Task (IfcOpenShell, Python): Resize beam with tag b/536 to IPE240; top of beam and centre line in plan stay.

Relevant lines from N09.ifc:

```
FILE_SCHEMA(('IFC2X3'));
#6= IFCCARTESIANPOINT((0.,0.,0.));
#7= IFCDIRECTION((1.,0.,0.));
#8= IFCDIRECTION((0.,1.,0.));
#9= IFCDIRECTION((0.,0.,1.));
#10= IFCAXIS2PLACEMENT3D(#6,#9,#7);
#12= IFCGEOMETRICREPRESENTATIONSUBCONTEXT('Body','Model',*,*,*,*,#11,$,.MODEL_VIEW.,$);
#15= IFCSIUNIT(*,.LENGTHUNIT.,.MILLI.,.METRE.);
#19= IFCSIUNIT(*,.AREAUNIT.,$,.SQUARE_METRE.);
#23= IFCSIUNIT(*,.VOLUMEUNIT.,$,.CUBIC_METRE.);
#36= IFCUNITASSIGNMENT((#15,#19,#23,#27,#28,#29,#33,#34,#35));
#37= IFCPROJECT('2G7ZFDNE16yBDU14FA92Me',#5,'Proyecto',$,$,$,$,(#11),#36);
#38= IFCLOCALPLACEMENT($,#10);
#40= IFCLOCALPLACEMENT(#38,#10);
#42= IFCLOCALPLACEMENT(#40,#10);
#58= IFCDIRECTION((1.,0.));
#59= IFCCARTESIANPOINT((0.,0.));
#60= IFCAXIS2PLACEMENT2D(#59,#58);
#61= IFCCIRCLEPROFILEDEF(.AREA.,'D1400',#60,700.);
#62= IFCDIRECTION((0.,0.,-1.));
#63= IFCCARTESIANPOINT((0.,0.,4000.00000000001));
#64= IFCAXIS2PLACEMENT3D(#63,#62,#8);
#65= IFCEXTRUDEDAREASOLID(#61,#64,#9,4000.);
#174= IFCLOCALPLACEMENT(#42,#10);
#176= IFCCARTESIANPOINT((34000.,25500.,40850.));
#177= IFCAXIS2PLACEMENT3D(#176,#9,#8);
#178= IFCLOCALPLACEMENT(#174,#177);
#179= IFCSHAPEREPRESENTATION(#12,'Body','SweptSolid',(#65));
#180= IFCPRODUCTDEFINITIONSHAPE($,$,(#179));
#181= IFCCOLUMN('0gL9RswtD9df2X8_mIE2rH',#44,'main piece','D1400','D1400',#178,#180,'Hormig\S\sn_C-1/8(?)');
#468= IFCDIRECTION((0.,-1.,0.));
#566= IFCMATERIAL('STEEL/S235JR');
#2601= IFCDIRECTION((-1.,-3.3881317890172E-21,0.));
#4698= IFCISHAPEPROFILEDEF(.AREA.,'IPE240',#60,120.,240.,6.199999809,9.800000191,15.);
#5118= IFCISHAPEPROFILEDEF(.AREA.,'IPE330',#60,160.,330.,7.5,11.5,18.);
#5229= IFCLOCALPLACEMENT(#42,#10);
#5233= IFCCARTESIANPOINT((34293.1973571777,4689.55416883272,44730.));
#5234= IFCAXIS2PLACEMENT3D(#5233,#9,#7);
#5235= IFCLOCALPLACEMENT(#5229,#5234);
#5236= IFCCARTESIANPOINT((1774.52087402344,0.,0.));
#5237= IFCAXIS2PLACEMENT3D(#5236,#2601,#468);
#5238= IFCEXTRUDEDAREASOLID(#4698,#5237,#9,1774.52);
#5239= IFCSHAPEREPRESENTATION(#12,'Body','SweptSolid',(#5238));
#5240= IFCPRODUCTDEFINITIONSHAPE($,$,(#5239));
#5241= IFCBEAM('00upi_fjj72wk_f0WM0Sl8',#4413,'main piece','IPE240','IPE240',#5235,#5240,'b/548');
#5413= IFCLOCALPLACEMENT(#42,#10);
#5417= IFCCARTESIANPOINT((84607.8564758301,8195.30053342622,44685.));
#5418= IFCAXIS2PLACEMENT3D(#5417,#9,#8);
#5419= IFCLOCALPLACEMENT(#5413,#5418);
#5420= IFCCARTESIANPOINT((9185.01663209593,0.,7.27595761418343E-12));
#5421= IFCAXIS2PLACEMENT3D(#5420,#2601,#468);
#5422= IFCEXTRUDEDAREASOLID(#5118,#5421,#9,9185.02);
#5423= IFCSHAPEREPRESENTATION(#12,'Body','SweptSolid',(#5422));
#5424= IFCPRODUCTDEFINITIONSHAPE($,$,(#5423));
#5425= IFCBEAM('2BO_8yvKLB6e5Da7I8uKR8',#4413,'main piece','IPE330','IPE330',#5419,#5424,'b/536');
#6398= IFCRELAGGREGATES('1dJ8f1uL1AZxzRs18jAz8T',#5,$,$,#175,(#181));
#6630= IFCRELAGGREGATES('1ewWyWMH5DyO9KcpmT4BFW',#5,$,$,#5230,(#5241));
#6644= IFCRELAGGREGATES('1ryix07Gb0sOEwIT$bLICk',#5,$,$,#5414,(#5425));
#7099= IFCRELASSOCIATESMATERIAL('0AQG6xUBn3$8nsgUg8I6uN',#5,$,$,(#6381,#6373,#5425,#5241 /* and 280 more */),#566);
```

```python
import ifcopenshell
import ifcopenshell.util.element
import ifcopenshell.util.representation

model = ifcopenshell.open("N09.ifc")

member = model.by_guid("2BO_8yvKLB6e5Da7I8uKR8")
source = next(p for p in model.by_type("IfcIShapeProfileDef") if p.ProfileName == "IPE240")

body = ifcopenshell.util.representation.get_representation(member, "Model", "Body")
solid = body.Items[0]
old_profile = solid.SweptArea

# Copy the section's sizes but keep this member's own profile position.
profile = ifcopenshell.util.element.copy(model, source)
# Profiles are centred, so shift by half the change in depth to hold the top.
shift = (old_profile.OverallDepth - profile.OverallDepth) / 2
x, y = old_profile.Position.Location.Coordinates
up = (0.0, 1.0)  # upwards, in the solid's own plane
location = model.createIfcCartesianPoint((x + up[0] * shift, y + up[1] * shift))
profile.Position = model.createIfcAxis2Placement2D(location, old_profile.Position.RefDirection)
solid.SweptArea = profile
if not model.get_total_inverses(old_profile):
    ifcopenshell.util.element.remove_deep2(model, old_profile)
member.Description = member.Description.replace("IPE330", "IPE240")
member.ObjectType = member.ObjectType.replace("IPE330", "IPE240")

print(solid.SweptArea)

model.write("N09_rev.ifc")
```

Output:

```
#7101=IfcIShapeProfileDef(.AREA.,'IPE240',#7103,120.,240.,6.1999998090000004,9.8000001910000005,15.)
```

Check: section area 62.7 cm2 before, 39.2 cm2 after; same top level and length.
